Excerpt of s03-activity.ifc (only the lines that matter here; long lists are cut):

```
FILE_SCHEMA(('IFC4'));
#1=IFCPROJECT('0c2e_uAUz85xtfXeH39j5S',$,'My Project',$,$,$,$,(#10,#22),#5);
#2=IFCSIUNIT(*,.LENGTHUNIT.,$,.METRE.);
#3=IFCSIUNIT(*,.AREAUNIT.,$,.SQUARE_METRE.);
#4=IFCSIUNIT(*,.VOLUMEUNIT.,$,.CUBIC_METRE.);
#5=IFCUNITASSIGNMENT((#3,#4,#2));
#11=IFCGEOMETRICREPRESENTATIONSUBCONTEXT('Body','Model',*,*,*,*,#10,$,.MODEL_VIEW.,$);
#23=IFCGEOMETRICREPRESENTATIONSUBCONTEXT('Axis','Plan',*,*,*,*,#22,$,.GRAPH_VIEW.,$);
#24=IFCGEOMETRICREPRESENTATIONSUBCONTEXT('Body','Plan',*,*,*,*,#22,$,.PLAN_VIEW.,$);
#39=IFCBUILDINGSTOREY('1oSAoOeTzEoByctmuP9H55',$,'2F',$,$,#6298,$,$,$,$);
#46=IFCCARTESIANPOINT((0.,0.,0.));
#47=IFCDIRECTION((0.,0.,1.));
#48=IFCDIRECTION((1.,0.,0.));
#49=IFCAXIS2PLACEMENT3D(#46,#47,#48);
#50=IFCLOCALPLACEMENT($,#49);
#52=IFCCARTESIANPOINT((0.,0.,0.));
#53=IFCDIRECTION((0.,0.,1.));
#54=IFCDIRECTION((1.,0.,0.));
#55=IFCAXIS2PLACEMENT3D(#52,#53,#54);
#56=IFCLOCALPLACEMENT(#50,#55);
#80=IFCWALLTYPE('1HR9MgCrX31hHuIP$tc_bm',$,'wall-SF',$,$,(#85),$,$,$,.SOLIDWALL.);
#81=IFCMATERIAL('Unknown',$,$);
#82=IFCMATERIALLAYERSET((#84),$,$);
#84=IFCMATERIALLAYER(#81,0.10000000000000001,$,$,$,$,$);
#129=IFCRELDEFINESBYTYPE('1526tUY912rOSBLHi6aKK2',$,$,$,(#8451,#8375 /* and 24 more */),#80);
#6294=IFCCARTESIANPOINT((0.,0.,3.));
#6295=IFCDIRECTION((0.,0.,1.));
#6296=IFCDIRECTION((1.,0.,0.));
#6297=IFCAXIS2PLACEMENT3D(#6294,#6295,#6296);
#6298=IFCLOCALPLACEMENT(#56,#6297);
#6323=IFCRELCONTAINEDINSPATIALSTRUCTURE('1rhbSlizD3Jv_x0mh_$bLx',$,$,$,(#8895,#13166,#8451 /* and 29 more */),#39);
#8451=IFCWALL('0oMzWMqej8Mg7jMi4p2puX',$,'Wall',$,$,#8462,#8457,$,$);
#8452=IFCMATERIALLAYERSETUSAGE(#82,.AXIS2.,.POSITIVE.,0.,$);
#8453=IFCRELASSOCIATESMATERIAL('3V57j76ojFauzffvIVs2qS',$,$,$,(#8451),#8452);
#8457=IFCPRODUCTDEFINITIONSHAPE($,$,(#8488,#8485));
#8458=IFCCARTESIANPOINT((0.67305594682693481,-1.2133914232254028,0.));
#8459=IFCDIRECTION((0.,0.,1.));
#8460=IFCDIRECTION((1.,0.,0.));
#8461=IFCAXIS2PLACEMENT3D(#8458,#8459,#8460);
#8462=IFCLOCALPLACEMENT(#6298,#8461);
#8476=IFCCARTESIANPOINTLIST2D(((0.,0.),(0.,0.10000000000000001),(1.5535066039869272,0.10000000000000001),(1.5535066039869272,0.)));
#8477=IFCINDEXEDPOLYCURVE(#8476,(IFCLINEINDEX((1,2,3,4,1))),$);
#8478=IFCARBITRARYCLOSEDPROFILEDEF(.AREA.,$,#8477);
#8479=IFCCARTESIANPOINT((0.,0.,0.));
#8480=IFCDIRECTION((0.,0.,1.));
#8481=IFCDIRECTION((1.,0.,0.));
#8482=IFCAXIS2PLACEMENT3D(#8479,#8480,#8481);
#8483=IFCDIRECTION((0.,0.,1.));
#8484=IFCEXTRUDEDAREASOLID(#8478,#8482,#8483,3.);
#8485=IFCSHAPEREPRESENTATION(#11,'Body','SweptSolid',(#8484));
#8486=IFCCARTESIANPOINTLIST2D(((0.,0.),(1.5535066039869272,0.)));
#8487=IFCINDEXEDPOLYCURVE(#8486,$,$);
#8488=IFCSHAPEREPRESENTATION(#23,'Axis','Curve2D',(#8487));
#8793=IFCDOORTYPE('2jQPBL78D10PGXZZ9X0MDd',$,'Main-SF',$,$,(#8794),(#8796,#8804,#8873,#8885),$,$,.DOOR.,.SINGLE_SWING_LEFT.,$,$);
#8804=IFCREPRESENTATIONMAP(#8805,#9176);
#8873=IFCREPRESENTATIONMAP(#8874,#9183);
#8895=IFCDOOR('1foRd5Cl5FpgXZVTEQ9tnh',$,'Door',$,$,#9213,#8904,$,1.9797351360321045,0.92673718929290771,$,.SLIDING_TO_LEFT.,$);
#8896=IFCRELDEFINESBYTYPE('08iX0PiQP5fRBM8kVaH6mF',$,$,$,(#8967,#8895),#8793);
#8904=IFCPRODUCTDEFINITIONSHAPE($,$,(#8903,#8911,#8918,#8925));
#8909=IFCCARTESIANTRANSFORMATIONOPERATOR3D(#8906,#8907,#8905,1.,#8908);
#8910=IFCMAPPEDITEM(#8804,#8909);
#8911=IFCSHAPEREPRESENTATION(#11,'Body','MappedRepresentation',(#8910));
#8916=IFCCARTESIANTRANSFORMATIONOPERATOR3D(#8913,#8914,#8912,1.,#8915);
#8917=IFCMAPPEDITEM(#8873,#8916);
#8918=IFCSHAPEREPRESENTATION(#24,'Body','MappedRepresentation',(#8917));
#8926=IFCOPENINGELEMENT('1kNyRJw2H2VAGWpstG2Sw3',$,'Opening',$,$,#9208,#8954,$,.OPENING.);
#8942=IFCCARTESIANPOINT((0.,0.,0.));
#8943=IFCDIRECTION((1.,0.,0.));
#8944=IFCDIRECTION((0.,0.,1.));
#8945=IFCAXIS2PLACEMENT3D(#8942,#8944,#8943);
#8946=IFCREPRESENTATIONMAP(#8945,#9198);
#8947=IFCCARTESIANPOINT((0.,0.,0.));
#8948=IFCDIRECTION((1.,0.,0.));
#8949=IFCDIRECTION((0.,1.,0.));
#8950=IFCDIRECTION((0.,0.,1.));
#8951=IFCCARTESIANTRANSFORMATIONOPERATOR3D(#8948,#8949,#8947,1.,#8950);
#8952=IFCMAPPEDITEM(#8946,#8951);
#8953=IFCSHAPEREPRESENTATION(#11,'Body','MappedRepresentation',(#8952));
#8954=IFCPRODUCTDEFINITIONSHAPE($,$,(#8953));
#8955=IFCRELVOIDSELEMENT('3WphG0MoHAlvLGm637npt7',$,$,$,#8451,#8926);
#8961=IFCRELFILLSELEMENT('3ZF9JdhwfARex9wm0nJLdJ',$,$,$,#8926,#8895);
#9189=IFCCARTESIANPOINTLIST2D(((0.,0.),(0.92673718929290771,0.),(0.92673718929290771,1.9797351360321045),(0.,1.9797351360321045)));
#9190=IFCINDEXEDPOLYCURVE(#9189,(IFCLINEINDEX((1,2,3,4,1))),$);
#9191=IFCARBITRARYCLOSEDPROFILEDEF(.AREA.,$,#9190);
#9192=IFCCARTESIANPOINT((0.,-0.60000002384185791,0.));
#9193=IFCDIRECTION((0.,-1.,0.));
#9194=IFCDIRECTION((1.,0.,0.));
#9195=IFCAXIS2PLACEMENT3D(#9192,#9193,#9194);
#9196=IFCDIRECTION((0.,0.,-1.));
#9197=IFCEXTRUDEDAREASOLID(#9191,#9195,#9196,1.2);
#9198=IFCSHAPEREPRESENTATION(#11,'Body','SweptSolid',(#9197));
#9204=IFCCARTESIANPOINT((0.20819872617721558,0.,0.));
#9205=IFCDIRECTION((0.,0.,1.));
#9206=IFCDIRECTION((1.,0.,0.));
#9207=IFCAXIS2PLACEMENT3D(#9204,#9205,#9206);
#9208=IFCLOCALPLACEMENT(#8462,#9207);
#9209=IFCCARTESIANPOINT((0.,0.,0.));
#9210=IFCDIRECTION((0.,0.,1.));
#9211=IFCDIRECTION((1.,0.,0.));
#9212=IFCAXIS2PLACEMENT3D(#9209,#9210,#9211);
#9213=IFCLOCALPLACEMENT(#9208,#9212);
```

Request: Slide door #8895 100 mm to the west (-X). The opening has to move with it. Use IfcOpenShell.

```python
import ifcopenshell
import ifcopenshell.api.geometry
import ifcopenshell.util.placement
import ifcopenshell.util.unit

model = ifcopenshell.open("s03-activity.ifc")
unit_scale = ifcopenshell.util.unit.calculate_unit_scale(model)

door = model.by_guid("1foRd5Cl5FpgXZVTEQ9tnh")
opening = door.FillsVoids[0].RelatingOpeningElement
wall = opening.VoidsElements[0].RelatingBuildingElement

wall_matrix = ifcopenshell.util.placement.get_local_placement(wall.ObjectPlacement)
shift = wall_matrix[:3, 0] * -0.1 / unit_scale
before = ifcopenshell.util.placement.get_local_placement(door.ObjectPlacement)[:3, 3].copy()

# The door is placed relative to its opening, so it follows when the opening moves.
matrix = ifcopenshell.util.placement.get_local_placement(opening.ObjectPlacement)
matrix[:3, 3] += shift
ifcopenshell.api.geometry.edit_object_placement(
    model, product=opening, matrix=matrix, is_si=False, should_transform_children=True
)

after = ifcopenshell.util.placement.get_local_placement(door.ObjectPlacement)[:3, 3]
print("door moved by", (after - before).round(3) + 0.0)

model.write("s03-activity_rev.ifc")
```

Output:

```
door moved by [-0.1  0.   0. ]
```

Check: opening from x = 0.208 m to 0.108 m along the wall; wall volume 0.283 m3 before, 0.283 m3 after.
